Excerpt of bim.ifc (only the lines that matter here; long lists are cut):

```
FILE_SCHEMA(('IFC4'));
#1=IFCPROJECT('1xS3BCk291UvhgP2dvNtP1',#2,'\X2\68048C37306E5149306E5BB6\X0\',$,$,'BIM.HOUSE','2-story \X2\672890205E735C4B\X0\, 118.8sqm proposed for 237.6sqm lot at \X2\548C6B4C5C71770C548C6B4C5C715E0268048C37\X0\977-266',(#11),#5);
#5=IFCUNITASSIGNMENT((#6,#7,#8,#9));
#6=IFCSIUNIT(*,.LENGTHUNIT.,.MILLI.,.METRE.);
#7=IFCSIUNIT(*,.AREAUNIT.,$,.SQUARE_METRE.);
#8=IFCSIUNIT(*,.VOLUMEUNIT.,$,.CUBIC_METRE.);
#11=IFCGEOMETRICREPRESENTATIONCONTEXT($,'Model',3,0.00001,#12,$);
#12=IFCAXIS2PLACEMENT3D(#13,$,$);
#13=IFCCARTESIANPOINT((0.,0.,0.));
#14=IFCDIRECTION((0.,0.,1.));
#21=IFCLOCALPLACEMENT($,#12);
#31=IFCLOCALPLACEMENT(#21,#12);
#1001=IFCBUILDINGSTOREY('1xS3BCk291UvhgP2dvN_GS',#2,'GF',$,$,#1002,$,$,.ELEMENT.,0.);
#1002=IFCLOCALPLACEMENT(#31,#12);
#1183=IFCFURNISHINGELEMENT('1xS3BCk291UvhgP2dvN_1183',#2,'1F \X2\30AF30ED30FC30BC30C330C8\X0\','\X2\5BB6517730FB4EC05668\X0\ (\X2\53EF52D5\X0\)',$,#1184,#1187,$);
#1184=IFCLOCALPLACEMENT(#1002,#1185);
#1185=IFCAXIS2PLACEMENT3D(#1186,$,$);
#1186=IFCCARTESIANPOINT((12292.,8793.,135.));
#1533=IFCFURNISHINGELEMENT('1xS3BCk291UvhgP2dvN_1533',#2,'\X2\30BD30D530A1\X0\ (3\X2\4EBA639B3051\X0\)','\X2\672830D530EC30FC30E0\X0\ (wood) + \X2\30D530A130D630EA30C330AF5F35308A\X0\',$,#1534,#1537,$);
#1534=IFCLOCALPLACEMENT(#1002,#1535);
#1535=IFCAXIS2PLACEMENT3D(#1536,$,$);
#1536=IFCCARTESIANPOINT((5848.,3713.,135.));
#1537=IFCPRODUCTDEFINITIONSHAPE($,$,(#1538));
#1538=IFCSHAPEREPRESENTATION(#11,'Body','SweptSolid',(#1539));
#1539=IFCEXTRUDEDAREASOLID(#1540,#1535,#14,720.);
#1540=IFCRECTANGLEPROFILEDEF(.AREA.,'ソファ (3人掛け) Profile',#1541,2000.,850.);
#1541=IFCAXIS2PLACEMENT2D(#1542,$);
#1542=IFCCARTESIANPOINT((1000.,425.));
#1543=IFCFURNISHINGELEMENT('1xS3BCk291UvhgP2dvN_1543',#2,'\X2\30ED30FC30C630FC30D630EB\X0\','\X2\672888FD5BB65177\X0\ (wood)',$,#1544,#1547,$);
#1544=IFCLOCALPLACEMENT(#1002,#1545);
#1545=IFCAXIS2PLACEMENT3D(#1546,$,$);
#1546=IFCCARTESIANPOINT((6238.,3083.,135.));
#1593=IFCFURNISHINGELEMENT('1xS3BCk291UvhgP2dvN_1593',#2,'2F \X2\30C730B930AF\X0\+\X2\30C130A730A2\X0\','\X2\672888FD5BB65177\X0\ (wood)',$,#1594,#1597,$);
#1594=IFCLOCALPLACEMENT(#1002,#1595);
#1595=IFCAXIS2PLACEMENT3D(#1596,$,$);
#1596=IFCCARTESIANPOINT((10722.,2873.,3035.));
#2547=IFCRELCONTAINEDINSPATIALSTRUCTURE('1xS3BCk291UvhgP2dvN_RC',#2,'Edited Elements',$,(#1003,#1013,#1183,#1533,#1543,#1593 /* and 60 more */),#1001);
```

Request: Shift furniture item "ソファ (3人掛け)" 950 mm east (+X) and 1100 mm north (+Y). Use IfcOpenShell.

```python
import ifcopenshell
import ifcopenshell.api.geometry
import ifcopenshell.util.placement
import ifcopenshell.util.unit

model = ifcopenshell.open("bim.ifc")
unit_scale = ifcopenshell.util.unit.calculate_unit_scale(model)

item = model.by_guid("1xS3BCk291UvhgP2dvN_1533")
matrix = ifcopenshell.util.placement.get_local_placement(item.ObjectPlacement)
matrix[0, 3] += 0.95 / unit_scale
matrix[1, 3] += 1.1 / unit_scale
ifcopenshell.api.geometry.edit_object_placement(model, product=item, matrix=matrix, is_si=False)

print(ifcopenshell.util.placement.get_local_placement(item.ObjectPlacement).round(3) + 0.0)

model.write("bim_edited.ifc")
```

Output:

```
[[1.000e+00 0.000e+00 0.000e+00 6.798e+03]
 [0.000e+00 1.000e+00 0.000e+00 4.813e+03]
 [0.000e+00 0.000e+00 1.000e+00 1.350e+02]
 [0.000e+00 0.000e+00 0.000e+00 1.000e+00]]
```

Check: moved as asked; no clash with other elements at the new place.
